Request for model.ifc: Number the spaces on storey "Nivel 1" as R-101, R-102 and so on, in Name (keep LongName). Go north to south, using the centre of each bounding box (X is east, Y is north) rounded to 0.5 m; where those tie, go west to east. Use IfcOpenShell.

First a look at what the model holds.

```python
import ifcopenshell
import ifcopenshell.util.element
import ifcopenshell.util.placement

model = ifcopenshell.open("model.ifc")
print(model.schema)
storey = next(s for s in model.by_type("IfcBuildingStorey") if s.Name == "Nivel 1")
spaces = [e for e in ifcopenshell.util.element.get_decomposition(storey) if e.is_a("IfcSpace")]
for e in sorted(spaces, key=lambda e: e.id()):
    origin = ifcopenshell.util.placement.get_local_placement(e.ObjectPlacement)[:3, 3]
    print(e.id(), e.Name, e.LongName, origin.round(2) + 0.0, sep=" | ")
```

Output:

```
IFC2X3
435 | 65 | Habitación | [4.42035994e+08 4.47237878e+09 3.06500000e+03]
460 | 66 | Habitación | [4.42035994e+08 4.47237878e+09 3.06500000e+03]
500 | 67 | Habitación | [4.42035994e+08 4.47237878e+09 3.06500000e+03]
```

```python
import ifcopenshell
import ifcopenshell.geom
import ifcopenshell.util.element
import ifcopenshell.util.shape

model = ifcopenshell.open("model.ifc")
settings = ifcopenshell.geom.settings()
settings.set("use-world-coords", True)


def centre(element):
    shape = ifcopenshell.geom.create_shape(settings, element)
    return ifcopenshell.util.shape.get_bbox_centroid(shape.geometry)


storey = next(s for s in model.by_type("IfcBuildingStorey") if s.Name == "Nivel 1")
spaces = [e for e in ifcopenshell.util.element.get_decomposition(storey) if e.is_a("IfcSpace")]

# Insertion points can sit at a corner or the storey origin, so sort by the geometry (in metres).
centres = {e: centre(e) for e in spaces}
spaces.sort(key=lambda e: (-round(centres[e][1] / 0.5), centres[e][0]))

for i, e in enumerate(spaces, start=1):
    number = f"R-1{i:02d}"
    e.Name = number
    print(e.id(), number)

model.write("model_rev.ifc")
```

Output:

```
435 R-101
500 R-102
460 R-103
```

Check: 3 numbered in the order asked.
